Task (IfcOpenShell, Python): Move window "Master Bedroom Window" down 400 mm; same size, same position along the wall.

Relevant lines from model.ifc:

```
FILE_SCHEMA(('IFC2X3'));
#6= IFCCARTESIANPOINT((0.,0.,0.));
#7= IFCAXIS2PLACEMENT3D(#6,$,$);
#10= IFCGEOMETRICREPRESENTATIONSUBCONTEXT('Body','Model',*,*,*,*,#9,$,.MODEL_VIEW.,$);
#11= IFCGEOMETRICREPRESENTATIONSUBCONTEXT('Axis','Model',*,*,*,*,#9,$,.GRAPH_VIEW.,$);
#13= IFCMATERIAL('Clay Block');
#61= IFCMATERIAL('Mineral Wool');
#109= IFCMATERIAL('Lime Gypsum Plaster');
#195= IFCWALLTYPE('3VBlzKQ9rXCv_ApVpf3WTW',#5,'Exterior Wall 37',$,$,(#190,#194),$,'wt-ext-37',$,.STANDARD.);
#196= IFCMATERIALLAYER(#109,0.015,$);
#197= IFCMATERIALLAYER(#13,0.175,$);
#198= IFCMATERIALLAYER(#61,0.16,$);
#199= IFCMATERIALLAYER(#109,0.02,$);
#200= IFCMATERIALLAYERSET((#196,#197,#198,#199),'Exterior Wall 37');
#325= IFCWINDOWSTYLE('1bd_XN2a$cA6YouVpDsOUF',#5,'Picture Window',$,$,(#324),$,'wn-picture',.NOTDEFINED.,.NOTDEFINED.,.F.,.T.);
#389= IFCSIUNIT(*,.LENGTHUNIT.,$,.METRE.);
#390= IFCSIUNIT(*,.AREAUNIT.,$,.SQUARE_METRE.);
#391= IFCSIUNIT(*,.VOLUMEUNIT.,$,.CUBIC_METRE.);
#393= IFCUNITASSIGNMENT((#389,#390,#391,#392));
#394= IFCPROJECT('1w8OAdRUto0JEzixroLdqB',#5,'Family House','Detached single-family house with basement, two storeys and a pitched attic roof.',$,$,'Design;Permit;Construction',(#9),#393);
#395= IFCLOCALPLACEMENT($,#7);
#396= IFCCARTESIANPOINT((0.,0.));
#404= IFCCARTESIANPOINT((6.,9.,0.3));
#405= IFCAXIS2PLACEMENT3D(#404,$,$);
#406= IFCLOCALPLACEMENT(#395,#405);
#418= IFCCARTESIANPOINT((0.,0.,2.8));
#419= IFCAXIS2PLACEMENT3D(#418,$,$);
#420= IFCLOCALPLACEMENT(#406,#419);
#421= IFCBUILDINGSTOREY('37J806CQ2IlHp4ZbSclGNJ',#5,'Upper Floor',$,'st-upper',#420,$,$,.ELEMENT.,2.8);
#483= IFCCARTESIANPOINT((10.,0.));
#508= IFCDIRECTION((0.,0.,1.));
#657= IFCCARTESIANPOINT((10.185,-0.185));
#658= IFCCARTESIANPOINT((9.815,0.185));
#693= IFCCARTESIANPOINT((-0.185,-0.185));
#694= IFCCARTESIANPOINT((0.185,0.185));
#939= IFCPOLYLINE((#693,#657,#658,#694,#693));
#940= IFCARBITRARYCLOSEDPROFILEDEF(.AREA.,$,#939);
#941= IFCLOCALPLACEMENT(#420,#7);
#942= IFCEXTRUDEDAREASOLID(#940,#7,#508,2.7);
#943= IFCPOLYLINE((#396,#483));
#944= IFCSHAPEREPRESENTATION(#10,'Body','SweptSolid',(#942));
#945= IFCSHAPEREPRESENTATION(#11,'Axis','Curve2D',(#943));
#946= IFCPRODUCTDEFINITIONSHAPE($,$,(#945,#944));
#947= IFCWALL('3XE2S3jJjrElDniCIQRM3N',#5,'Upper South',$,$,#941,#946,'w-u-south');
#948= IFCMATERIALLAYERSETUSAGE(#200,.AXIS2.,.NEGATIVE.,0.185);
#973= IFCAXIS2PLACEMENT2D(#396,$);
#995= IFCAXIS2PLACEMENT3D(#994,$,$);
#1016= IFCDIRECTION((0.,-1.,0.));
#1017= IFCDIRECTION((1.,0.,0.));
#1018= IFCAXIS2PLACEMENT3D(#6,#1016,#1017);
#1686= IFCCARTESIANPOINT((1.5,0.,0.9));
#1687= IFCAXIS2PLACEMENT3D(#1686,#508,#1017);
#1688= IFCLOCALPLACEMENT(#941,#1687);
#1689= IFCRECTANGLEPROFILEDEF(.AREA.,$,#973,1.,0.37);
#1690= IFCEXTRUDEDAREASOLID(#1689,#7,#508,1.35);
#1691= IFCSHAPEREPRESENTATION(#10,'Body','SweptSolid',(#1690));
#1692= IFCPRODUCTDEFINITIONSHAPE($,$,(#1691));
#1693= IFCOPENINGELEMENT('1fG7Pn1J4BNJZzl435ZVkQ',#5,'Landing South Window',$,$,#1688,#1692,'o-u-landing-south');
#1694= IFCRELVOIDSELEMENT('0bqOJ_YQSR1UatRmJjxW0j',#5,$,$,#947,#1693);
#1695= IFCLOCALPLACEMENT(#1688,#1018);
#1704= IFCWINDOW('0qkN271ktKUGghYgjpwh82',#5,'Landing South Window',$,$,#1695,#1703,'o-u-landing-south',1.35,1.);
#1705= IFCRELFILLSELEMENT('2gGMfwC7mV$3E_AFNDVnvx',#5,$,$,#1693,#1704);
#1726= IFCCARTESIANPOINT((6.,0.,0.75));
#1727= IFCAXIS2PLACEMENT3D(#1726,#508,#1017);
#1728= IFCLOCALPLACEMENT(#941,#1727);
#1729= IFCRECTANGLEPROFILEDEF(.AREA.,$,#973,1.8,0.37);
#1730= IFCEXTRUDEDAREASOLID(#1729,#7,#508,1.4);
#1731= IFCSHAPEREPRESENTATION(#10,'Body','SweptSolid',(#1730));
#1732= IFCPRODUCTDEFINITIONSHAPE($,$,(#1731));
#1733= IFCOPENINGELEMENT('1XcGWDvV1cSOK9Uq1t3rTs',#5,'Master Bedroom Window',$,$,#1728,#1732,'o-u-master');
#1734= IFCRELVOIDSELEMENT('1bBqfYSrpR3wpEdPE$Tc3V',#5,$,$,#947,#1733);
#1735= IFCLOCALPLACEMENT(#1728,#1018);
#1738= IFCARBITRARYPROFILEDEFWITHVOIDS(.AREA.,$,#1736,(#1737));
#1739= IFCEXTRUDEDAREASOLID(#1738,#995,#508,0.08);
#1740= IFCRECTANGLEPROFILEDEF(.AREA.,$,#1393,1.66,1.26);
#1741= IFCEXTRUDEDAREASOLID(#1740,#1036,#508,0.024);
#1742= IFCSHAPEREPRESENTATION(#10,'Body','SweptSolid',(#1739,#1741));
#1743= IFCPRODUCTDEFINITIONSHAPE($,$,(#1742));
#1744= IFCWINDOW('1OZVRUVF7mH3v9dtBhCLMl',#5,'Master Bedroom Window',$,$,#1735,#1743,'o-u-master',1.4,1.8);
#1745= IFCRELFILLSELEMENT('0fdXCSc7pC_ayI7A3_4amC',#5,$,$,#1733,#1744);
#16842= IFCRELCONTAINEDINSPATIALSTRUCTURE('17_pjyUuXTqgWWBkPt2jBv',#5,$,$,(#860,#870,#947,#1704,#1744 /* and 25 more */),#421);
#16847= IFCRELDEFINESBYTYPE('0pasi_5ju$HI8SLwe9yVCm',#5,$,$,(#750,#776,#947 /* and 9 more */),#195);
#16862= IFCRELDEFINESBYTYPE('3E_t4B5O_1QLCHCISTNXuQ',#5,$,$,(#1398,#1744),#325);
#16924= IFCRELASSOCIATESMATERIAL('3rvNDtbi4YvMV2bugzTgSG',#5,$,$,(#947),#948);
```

```python
import numpy as np
import ifcopenshell
import ifcopenshell.api.geometry
import ifcopenshell.util.placement
import ifcopenshell.util.unit

model = ifcopenshell.open("model.ifc")
unit_scale = ifcopenshell.util.unit.calculate_unit_scale(model)

window = model.by_guid("1OZVRUVF7mH3v9dtBhCLMl")
opening = window.FillsVoids[0].RelatingOpeningElement
dz = -0.4 / unit_scale

shift = np.array([0.0, 0.0, dz])
# The window is placed relative to its opening, so it follows when the opening moves.
matrix = ifcopenshell.util.placement.get_local_placement(opening.ObjectPlacement)
matrix[:3, 3] += shift
ifcopenshell.api.geometry.edit_object_placement(
    model, product=opening, matrix=matrix, is_si=False, should_transform_children=True
)

print(f"moved by {dz * unit_scale:+.3f} m")

model.write("model_rev.ifc")
```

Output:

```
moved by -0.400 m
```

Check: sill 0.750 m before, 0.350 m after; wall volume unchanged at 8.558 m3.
